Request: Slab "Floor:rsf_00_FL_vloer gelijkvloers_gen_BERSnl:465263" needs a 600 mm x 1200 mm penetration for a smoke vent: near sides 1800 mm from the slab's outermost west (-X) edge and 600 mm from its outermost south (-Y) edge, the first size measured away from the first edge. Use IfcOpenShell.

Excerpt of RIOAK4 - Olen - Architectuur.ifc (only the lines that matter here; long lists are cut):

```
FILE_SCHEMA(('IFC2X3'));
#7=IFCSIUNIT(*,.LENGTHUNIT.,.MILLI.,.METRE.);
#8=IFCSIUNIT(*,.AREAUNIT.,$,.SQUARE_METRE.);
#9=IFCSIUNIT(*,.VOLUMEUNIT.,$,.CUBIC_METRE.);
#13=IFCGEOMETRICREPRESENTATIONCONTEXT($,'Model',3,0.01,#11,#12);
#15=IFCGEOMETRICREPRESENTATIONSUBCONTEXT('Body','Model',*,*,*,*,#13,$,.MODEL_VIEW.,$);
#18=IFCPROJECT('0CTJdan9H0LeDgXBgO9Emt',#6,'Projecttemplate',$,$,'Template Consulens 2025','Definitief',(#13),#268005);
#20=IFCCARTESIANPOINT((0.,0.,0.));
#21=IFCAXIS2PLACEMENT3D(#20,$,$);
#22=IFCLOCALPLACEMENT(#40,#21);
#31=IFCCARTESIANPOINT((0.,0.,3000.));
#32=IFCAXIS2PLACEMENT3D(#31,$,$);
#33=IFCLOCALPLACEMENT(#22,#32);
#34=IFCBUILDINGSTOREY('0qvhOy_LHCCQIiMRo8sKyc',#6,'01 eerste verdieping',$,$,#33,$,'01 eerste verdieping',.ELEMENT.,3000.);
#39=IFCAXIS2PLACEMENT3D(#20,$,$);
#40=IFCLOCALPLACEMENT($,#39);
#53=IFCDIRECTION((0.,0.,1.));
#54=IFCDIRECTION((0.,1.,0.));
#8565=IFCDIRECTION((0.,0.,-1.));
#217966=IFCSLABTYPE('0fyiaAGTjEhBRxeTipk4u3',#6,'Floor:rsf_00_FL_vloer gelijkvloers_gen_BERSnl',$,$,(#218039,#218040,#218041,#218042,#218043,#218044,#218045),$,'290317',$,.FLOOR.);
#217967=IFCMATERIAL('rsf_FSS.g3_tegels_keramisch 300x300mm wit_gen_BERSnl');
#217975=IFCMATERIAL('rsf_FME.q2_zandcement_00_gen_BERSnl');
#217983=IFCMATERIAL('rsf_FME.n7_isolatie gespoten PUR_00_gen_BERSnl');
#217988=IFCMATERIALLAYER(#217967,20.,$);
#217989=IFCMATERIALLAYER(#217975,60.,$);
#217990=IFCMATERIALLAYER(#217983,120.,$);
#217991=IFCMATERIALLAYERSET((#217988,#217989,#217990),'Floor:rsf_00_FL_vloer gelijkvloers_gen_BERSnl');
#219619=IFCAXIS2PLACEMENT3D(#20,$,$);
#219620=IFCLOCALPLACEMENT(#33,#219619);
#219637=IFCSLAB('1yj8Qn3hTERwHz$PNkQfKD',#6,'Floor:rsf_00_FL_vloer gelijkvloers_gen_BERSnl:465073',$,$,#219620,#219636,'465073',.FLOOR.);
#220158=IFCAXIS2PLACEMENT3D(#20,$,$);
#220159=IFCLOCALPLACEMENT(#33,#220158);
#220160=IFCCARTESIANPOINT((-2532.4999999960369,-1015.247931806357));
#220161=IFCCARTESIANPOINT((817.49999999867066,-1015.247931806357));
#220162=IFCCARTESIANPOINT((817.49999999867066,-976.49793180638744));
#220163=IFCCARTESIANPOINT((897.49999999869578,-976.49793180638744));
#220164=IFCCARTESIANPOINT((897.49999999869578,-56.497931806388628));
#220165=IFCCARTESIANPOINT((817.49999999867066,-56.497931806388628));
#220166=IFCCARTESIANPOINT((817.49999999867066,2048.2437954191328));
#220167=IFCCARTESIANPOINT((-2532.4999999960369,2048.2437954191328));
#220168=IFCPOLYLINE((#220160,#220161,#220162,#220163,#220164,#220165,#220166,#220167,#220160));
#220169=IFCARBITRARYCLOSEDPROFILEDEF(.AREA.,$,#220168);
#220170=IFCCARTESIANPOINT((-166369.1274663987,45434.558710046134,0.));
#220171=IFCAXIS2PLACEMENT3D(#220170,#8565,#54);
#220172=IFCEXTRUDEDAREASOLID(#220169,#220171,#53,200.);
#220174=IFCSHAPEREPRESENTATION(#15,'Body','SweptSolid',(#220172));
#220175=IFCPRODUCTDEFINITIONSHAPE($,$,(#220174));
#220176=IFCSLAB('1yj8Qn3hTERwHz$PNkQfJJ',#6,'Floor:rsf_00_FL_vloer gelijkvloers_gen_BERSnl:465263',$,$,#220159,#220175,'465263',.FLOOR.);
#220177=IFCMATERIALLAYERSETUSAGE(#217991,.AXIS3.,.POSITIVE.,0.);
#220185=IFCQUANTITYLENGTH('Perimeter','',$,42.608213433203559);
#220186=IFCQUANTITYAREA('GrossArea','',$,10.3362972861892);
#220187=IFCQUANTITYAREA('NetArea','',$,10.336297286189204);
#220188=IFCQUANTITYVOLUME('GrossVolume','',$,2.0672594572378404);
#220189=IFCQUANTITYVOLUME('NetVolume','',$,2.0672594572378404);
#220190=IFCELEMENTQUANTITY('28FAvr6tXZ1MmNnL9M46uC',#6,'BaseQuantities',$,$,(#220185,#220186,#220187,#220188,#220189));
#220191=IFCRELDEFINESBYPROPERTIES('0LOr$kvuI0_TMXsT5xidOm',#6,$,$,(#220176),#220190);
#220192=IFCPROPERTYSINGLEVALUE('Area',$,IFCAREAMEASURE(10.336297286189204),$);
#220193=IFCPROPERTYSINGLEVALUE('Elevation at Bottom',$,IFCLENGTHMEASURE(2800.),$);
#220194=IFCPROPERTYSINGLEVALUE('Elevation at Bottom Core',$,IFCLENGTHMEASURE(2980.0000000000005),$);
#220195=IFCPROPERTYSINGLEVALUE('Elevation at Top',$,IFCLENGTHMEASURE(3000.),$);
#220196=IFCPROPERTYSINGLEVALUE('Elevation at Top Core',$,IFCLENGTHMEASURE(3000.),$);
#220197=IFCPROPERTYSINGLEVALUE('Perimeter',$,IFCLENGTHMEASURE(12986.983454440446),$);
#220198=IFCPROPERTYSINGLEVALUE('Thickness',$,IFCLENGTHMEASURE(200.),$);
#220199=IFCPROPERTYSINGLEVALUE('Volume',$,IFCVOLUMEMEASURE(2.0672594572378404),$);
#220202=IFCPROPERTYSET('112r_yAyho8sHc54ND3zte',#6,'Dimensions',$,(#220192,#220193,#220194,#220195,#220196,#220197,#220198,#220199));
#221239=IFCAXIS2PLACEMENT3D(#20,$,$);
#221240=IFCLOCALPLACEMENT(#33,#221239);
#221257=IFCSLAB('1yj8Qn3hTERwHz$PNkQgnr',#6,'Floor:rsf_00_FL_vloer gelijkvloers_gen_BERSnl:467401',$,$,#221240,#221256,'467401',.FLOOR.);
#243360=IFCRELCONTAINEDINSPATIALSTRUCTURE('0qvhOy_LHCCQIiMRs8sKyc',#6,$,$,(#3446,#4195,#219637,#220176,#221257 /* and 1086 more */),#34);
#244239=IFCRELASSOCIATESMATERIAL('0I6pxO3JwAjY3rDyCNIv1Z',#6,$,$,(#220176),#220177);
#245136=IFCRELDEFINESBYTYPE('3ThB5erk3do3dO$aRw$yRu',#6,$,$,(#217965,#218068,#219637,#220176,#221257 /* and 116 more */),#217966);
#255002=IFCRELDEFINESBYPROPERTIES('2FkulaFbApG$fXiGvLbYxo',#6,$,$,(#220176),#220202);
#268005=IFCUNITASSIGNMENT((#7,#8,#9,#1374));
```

```python
import numpy as np
import ifcopenshell
import ifcopenshell.api.feature
import ifcopenshell.api.geometry
import ifcopenshell.api.pset
import ifcopenshell.api.root
import ifcopenshell.geom
import ifcopenshell.util.element
import ifcopenshell.util.placement
import ifcopenshell.util.representation
import ifcopenshell.util.shape
import ifcopenshell.util.unit

model = ifcopenshell.open("RIOAK4 - Olen - Architectuur.ifc")
unit_scale = ifcopenshell.util.unit.calculate_unit_scale(model)
area_scale = ifcopenshell.util.unit.calculate_unit_scale(model, "AREAUNIT")
volume_scale = ifcopenshell.util.unit.calculate_unit_scale(model, "VOLUMEUNIT")
settings = ifcopenshell.geom.settings()


def volume(element):
    """Net volume in cubic metres, openings subtracted."""
    shape = ifcopenshell.geom.create_shape(settings, element)
    return ifcopenshell.util.shape.get_volume(shape.geometry)


slab = model.by_id(220176)
before = volume(slab)

# Extent in the slab's own axes, in metres. The edges named are its -X and -Y sides.
slab_shape = ifcopenshell.geom.create_shape(settings, slab)
vertices = ifcopenshell.util.shape.get_vertices(slab_shape.geometry)
x_min, y_min, bottom = vertices.min(axis=0)
top = vertices[:, 2].max()

opening = ifcopenshell.api.root.create_entity(model, ifc_class="IfcOpeningElement", name="Smoke vent opening")
context = ifcopenshell.util.representation.get_context(model, "Model", "Body", "MODEL_VIEW")
width, depth = 0.6, 1.2
outline = [(0.0, 0.0), (width, 0.0), (width, depth), (0.0, depth), (0.0, 0.0)]
# Overshoot both faces by 50 mm so the cut is clean.
shape = ifcopenshell.api.geometry.add_slab_representation(
    model, context=context, depth=top - bottom + 0.1, polyline=outline
)
ifcopenshell.api.geometry.assign_representation(model, product=opening, representation=shape)

matrix = ifcopenshell.util.placement.get_local_placement(slab.ObjectPlacement)
matrix[:, 3] = matrix @ np.append(np.array([x_min + 1.8, y_min + 0.6, bottom - 0.05]) / unit_scale, 1.0)
ifcopenshell.api.geometry.edit_object_placement(model, product=opening, matrix=matrix, is_si=False)
ifcopenshell.api.feature.add_feature(model, feature=opening, element=slab)

after = volume(slab)

# Update the slab's stored quantities.
qto = model.by_id(ifcopenshell.util.element.get_pset(slab, "BaseQuantities", should_inherit=False)["id"])
ifcopenshell.api.pset.edit_qto(model, qto=qto, properties={
    "NetArea": after / (top - bottom) / area_scale,
    "NetVolume": after / volume_scale,
})
pset = model.by_id(ifcopenshell.util.element.get_pset(slab, "Dimensions", should_inherit=False)["id"])
ifcopenshell.api.pset.edit_pset(model, pset=pset, properties={
    "Area": model.create_entity("IfcAreaMeasure", after / (top - bottom) / area_scale),
    "Volume": model.create_entity("IfcVolumeMeasure", after / volume_scale),
})

print(f"slab volume {before:.3f} -> {after:.3f} m3")

model.write("RIOAK4 - Olen - Architectuur_v2.ifc")
```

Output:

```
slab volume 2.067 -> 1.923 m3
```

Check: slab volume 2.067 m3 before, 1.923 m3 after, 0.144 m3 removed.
